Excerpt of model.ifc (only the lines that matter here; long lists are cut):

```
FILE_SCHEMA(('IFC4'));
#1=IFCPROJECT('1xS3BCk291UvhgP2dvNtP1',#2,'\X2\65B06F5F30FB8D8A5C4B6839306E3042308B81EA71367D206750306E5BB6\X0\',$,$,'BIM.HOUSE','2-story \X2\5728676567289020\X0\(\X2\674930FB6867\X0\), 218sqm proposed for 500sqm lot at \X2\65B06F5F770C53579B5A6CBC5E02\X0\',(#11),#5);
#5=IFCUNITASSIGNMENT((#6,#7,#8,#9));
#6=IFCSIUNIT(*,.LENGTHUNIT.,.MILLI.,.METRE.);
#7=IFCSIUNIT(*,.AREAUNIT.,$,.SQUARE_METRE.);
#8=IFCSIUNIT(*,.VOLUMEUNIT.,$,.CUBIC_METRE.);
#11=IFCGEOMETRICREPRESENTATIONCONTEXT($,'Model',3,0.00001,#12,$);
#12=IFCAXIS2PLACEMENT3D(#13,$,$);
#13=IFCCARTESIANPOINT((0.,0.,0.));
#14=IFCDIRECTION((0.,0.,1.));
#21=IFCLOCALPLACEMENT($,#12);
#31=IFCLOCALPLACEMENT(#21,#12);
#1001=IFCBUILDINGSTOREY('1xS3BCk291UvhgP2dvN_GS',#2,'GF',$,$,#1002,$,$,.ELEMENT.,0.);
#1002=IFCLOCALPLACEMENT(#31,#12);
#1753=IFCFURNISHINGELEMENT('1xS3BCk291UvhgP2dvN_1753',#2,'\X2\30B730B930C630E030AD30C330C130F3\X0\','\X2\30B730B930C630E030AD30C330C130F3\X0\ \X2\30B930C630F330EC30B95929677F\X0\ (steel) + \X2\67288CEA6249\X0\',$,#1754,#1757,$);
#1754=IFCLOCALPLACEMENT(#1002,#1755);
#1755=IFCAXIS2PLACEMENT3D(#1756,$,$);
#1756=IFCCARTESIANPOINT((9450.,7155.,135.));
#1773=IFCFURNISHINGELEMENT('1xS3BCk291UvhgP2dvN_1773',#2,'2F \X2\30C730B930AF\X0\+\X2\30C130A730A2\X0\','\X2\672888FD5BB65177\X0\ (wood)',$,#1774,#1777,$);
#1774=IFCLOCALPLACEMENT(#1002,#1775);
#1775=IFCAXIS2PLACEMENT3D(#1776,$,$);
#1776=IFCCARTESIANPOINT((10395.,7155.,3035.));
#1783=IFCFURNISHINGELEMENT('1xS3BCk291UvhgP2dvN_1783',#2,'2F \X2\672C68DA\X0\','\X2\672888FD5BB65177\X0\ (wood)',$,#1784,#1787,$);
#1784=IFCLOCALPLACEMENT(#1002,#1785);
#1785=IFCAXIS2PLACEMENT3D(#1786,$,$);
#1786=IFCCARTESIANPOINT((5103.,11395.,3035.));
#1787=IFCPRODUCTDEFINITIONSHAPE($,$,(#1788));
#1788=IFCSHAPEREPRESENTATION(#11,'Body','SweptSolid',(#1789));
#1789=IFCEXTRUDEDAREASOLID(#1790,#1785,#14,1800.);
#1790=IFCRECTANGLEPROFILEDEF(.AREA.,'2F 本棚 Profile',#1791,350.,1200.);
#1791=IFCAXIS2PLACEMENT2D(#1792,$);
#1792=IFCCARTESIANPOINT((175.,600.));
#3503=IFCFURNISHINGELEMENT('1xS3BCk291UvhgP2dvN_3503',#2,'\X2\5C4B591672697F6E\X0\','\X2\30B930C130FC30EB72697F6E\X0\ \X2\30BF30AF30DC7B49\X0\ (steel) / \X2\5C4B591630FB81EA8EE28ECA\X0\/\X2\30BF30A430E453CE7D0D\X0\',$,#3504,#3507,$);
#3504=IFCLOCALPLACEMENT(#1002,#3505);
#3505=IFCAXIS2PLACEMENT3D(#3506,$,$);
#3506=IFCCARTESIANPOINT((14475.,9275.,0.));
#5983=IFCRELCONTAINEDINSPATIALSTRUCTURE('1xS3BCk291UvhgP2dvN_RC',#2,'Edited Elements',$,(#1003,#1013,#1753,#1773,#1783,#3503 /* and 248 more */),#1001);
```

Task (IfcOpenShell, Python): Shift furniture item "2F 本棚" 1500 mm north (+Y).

```python
import ifcopenshell
import ifcopenshell.api.geometry
import ifcopenshell.util.placement
import ifcopenshell.util.unit

model = ifcopenshell.open("model.ifc")
unit_scale = ifcopenshell.util.unit.calculate_unit_scale(model)

item = model.by_id(1783)
matrix = ifcopenshell.util.placement.get_local_placement(item.ObjectPlacement)
matrix[1, 3] += 1.5 / unit_scale
ifcopenshell.api.geometry.edit_object_placement(model, product=item, matrix=matrix, is_si=False)

print(ifcopenshell.util.placement.get_local_placement(item.ObjectPlacement).round(3) + 0.0)

model.write("model_rev.ifc")
```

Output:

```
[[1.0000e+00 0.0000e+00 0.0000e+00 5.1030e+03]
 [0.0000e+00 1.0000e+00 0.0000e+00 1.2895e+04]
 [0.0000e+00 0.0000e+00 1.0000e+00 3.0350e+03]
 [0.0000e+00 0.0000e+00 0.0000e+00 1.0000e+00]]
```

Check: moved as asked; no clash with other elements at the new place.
